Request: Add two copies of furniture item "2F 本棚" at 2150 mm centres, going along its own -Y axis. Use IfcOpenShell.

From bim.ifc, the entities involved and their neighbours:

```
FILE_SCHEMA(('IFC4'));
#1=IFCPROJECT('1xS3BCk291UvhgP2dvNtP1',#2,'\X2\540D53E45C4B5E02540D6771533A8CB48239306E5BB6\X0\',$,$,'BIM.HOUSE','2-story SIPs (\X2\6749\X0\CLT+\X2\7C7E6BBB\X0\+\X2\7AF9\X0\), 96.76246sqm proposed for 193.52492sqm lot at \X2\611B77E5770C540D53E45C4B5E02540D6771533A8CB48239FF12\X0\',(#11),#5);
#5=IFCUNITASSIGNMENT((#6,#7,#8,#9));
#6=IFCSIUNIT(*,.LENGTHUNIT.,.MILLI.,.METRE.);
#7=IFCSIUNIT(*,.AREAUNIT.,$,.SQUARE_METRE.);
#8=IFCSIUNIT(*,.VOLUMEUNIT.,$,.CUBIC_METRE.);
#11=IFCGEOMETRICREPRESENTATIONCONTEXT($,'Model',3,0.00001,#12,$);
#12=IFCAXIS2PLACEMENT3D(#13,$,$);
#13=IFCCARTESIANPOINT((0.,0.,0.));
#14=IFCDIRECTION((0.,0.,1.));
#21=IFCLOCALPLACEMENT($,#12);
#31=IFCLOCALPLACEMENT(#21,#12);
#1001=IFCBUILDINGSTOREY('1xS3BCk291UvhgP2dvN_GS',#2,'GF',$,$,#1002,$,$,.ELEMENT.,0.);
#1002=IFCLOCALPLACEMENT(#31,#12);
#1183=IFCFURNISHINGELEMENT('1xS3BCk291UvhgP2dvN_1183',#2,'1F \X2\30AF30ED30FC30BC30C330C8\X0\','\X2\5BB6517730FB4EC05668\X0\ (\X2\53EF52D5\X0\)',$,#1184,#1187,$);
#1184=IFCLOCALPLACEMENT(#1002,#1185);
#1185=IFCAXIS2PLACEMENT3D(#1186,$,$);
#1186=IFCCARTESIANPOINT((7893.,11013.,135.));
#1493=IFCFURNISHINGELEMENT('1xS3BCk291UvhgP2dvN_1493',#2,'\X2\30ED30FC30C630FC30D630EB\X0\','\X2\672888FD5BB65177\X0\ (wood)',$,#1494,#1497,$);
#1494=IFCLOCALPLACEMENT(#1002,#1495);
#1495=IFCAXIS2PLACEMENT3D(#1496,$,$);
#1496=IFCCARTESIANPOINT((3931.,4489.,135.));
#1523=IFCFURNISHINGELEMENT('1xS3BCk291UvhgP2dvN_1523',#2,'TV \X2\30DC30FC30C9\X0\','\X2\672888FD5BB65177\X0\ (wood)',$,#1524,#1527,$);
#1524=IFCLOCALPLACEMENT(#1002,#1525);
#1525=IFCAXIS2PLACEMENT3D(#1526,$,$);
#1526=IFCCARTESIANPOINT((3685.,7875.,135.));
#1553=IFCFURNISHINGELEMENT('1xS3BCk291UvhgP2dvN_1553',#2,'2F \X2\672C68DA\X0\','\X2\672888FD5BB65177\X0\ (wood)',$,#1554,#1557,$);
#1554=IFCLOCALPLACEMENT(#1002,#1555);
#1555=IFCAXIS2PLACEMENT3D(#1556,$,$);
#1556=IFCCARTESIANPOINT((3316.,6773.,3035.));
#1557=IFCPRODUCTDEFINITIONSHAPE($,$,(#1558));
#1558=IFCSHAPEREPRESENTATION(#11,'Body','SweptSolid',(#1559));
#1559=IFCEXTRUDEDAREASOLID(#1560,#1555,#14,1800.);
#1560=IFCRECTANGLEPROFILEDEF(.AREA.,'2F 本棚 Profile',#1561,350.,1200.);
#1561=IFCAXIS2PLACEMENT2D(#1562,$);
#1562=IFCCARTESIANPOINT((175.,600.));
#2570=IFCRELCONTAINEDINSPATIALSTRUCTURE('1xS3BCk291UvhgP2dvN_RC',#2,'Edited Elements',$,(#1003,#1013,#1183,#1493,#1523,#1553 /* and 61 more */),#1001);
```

```python
import ifcopenshell
import ifcopenshell.api.geometry
import ifcopenshell.api.root
import ifcopenshell.util.element
import ifcopenshell.util.placement

model = ifcopenshell.open("bim.ifc")


def reuse_history(source, copy):
    """copy_class also copies each property set's owner history, people and application; keep the originals."""
    for rel in copy.IsDefinedBy:
        if rel.is_a("IfcRelDefinesByProperties") and (history := rel.RelatingPropertyDefinition.OwnerHistory):
            rel.RelatingPropertyDefinition.OwnerHistory = source.OwnerHistory
            ifcopenshell.util.element.remove_deep2(model, history)


source = model.by_id(1553)
base = ifcopenshell.util.placement.get_local_placement(source.ObjectPlacement)
step = -base[:3, 1] * 2150.0

for i in range(1, 3):
    copy = ifcopenshell.api.root.copy_class(model, product=source)
    copy.Representation = ifcopenshell.util.element.copy_deep(
        model, source.Representation, exclude=["IfcGeometricRepresentationContext", "IfcRepresentationMap"]
    )
    reuse_history(source, copy)
    matrix = base.copy()
    matrix[:3, 3] += i * step
    print("added at", matrix[:3, 3].round(3) + 0.0)
    ifcopenshell.api.geometry.edit_object_placement(model, product=copy, matrix=matrix, is_si=False)

model.write("bim_edited.ifc")
```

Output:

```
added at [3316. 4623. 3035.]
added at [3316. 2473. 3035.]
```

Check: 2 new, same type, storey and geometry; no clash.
